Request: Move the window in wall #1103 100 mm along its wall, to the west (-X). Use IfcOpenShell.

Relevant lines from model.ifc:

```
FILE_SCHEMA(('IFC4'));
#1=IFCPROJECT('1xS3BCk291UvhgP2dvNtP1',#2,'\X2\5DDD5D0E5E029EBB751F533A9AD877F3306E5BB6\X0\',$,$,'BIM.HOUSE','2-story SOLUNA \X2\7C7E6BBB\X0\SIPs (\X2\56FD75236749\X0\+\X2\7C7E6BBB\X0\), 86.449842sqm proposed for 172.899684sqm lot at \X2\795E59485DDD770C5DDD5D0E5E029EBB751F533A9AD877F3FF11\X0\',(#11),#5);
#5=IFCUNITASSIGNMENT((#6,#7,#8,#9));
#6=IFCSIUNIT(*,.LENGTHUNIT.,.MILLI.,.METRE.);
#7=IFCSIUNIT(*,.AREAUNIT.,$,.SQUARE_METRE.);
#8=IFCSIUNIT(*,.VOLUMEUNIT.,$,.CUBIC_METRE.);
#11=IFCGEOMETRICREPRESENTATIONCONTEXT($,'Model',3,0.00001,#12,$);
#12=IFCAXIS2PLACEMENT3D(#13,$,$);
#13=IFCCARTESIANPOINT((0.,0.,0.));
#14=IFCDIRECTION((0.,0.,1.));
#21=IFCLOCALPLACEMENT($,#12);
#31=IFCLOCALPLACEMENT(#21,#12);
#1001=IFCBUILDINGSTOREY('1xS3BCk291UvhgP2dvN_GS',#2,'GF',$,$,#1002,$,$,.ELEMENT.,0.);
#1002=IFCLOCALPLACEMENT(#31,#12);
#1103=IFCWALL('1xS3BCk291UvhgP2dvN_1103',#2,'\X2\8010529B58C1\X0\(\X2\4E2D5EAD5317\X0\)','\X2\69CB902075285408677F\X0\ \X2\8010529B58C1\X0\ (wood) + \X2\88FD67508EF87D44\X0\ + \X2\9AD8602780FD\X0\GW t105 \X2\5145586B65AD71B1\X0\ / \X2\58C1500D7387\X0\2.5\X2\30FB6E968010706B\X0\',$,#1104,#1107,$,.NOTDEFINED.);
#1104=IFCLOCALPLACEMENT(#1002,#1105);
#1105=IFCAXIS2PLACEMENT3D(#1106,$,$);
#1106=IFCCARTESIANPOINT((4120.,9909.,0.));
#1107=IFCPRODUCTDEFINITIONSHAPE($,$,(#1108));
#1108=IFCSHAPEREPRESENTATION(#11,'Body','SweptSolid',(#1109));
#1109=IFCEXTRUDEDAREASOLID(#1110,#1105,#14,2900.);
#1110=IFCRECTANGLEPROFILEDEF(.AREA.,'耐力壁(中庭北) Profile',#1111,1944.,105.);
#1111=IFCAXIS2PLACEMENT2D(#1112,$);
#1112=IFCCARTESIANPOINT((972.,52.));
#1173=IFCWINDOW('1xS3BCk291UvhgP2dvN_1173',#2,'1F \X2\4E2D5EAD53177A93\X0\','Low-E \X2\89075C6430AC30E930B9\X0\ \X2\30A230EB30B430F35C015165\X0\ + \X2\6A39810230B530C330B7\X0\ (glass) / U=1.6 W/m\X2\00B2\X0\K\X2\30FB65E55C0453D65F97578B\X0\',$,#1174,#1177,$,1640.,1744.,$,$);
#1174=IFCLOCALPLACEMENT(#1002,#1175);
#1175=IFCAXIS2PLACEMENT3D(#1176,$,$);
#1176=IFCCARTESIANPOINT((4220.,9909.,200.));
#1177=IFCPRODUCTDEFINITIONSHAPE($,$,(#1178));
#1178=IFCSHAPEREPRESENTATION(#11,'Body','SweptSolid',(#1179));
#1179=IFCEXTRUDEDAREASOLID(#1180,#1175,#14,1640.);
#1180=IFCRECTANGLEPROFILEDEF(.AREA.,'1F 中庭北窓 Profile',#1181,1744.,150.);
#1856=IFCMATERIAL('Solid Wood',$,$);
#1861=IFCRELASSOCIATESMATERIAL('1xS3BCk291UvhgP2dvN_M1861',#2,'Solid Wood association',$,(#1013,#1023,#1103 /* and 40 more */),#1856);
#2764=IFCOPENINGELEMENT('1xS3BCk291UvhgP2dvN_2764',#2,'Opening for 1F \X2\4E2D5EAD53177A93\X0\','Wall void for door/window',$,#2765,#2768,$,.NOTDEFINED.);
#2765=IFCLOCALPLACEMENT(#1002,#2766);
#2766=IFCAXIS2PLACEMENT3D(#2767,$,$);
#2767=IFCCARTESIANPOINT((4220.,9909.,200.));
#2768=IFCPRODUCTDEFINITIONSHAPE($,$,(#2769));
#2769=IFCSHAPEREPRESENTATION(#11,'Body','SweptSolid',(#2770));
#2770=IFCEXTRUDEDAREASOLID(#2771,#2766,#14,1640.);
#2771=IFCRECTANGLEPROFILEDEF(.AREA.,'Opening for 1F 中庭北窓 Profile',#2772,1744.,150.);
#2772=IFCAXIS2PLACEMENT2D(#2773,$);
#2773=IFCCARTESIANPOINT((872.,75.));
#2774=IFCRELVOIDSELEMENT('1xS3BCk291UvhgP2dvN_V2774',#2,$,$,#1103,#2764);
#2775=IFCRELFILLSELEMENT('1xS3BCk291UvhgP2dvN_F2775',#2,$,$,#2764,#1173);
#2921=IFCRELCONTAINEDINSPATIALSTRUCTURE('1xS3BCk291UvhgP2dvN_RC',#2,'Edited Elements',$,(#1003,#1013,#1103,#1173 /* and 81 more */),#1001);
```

```python
import ifcopenshell
import ifcopenshell.api.geometry
import ifcopenshell.util.placement
import ifcopenshell.util.unit

model = ifcopenshell.open("model.ifc")
unit_scale = ifcopenshell.util.unit.calculate_unit_scale(model)

window = model.by_guid("1xS3BCk291UvhgP2dvN_1173")
opening = window.FillsVoids[0].RelatingOpeningElement
wall = opening.VoidsElements[0].RelatingBuildingElement

wall_matrix = ifcopenshell.util.placement.get_local_placement(wall.ObjectPlacement)
shift = wall_matrix[:3, 0] * -0.1 / unit_scale
before = ifcopenshell.util.placement.get_local_placement(window.ObjectPlacement)[:3, 3].copy()

# The window is not placed relative to its opening, so move both.
for product in (opening, window):
    matrix = ifcopenshell.util.placement.get_local_placement(product.ObjectPlacement)
    matrix[:3, 3] += shift
    ifcopenshell.api.geometry.edit_object_placement(model, product=product, matrix=matrix, is_si=False)

after = ifcopenshell.util.placement.get_local_placement(window.ObjectPlacement)[:3, 3]
print("window moved by", (after - before).round(3) + 0.0)

model.write("model_rev.ifc")
```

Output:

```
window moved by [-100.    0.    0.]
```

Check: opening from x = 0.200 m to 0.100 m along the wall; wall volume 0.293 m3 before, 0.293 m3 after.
